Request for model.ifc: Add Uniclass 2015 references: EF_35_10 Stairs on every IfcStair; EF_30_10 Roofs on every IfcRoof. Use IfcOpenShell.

First a look at what the model holds.

```python
import ifcopenshell

model = ifcopenshell.open("model.ifc")
print(model.schema)
print("classifications:", [c.Name for c in model.by_type("IfcClassification")])
for ifc_class in ("IfcDoor", "IfcRoof", "IfcStair", "IfcWall", "IfcWindow"):
    print(ifc_class, len(model.by_type(ifc_class)))
```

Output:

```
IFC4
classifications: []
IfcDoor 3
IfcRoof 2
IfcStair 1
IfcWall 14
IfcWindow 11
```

```python
import ifcopenshell
import ifcopenshell.api.classification

model = ifcopenshell.open("model.ifc")

system = ifcopenshell.api.classification.add_classification(model, classification="Uniclass 2015")

codes = {
    "IfcStair": ("EF_35_10", "Stairs"),
    "IfcRoof": ("EF_30_10", "Roofs"),
}
for ifc_class, (code, name) in codes.items():
    products = model.by_type(ifc_class)
    ifcopenshell.api.classification.add_reference(
        model, products=products, classification=system, identification=code, name=name
    )
    print(code, len(products))

model.write("model_edited.ifc")
```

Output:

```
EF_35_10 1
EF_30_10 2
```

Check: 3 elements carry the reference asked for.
